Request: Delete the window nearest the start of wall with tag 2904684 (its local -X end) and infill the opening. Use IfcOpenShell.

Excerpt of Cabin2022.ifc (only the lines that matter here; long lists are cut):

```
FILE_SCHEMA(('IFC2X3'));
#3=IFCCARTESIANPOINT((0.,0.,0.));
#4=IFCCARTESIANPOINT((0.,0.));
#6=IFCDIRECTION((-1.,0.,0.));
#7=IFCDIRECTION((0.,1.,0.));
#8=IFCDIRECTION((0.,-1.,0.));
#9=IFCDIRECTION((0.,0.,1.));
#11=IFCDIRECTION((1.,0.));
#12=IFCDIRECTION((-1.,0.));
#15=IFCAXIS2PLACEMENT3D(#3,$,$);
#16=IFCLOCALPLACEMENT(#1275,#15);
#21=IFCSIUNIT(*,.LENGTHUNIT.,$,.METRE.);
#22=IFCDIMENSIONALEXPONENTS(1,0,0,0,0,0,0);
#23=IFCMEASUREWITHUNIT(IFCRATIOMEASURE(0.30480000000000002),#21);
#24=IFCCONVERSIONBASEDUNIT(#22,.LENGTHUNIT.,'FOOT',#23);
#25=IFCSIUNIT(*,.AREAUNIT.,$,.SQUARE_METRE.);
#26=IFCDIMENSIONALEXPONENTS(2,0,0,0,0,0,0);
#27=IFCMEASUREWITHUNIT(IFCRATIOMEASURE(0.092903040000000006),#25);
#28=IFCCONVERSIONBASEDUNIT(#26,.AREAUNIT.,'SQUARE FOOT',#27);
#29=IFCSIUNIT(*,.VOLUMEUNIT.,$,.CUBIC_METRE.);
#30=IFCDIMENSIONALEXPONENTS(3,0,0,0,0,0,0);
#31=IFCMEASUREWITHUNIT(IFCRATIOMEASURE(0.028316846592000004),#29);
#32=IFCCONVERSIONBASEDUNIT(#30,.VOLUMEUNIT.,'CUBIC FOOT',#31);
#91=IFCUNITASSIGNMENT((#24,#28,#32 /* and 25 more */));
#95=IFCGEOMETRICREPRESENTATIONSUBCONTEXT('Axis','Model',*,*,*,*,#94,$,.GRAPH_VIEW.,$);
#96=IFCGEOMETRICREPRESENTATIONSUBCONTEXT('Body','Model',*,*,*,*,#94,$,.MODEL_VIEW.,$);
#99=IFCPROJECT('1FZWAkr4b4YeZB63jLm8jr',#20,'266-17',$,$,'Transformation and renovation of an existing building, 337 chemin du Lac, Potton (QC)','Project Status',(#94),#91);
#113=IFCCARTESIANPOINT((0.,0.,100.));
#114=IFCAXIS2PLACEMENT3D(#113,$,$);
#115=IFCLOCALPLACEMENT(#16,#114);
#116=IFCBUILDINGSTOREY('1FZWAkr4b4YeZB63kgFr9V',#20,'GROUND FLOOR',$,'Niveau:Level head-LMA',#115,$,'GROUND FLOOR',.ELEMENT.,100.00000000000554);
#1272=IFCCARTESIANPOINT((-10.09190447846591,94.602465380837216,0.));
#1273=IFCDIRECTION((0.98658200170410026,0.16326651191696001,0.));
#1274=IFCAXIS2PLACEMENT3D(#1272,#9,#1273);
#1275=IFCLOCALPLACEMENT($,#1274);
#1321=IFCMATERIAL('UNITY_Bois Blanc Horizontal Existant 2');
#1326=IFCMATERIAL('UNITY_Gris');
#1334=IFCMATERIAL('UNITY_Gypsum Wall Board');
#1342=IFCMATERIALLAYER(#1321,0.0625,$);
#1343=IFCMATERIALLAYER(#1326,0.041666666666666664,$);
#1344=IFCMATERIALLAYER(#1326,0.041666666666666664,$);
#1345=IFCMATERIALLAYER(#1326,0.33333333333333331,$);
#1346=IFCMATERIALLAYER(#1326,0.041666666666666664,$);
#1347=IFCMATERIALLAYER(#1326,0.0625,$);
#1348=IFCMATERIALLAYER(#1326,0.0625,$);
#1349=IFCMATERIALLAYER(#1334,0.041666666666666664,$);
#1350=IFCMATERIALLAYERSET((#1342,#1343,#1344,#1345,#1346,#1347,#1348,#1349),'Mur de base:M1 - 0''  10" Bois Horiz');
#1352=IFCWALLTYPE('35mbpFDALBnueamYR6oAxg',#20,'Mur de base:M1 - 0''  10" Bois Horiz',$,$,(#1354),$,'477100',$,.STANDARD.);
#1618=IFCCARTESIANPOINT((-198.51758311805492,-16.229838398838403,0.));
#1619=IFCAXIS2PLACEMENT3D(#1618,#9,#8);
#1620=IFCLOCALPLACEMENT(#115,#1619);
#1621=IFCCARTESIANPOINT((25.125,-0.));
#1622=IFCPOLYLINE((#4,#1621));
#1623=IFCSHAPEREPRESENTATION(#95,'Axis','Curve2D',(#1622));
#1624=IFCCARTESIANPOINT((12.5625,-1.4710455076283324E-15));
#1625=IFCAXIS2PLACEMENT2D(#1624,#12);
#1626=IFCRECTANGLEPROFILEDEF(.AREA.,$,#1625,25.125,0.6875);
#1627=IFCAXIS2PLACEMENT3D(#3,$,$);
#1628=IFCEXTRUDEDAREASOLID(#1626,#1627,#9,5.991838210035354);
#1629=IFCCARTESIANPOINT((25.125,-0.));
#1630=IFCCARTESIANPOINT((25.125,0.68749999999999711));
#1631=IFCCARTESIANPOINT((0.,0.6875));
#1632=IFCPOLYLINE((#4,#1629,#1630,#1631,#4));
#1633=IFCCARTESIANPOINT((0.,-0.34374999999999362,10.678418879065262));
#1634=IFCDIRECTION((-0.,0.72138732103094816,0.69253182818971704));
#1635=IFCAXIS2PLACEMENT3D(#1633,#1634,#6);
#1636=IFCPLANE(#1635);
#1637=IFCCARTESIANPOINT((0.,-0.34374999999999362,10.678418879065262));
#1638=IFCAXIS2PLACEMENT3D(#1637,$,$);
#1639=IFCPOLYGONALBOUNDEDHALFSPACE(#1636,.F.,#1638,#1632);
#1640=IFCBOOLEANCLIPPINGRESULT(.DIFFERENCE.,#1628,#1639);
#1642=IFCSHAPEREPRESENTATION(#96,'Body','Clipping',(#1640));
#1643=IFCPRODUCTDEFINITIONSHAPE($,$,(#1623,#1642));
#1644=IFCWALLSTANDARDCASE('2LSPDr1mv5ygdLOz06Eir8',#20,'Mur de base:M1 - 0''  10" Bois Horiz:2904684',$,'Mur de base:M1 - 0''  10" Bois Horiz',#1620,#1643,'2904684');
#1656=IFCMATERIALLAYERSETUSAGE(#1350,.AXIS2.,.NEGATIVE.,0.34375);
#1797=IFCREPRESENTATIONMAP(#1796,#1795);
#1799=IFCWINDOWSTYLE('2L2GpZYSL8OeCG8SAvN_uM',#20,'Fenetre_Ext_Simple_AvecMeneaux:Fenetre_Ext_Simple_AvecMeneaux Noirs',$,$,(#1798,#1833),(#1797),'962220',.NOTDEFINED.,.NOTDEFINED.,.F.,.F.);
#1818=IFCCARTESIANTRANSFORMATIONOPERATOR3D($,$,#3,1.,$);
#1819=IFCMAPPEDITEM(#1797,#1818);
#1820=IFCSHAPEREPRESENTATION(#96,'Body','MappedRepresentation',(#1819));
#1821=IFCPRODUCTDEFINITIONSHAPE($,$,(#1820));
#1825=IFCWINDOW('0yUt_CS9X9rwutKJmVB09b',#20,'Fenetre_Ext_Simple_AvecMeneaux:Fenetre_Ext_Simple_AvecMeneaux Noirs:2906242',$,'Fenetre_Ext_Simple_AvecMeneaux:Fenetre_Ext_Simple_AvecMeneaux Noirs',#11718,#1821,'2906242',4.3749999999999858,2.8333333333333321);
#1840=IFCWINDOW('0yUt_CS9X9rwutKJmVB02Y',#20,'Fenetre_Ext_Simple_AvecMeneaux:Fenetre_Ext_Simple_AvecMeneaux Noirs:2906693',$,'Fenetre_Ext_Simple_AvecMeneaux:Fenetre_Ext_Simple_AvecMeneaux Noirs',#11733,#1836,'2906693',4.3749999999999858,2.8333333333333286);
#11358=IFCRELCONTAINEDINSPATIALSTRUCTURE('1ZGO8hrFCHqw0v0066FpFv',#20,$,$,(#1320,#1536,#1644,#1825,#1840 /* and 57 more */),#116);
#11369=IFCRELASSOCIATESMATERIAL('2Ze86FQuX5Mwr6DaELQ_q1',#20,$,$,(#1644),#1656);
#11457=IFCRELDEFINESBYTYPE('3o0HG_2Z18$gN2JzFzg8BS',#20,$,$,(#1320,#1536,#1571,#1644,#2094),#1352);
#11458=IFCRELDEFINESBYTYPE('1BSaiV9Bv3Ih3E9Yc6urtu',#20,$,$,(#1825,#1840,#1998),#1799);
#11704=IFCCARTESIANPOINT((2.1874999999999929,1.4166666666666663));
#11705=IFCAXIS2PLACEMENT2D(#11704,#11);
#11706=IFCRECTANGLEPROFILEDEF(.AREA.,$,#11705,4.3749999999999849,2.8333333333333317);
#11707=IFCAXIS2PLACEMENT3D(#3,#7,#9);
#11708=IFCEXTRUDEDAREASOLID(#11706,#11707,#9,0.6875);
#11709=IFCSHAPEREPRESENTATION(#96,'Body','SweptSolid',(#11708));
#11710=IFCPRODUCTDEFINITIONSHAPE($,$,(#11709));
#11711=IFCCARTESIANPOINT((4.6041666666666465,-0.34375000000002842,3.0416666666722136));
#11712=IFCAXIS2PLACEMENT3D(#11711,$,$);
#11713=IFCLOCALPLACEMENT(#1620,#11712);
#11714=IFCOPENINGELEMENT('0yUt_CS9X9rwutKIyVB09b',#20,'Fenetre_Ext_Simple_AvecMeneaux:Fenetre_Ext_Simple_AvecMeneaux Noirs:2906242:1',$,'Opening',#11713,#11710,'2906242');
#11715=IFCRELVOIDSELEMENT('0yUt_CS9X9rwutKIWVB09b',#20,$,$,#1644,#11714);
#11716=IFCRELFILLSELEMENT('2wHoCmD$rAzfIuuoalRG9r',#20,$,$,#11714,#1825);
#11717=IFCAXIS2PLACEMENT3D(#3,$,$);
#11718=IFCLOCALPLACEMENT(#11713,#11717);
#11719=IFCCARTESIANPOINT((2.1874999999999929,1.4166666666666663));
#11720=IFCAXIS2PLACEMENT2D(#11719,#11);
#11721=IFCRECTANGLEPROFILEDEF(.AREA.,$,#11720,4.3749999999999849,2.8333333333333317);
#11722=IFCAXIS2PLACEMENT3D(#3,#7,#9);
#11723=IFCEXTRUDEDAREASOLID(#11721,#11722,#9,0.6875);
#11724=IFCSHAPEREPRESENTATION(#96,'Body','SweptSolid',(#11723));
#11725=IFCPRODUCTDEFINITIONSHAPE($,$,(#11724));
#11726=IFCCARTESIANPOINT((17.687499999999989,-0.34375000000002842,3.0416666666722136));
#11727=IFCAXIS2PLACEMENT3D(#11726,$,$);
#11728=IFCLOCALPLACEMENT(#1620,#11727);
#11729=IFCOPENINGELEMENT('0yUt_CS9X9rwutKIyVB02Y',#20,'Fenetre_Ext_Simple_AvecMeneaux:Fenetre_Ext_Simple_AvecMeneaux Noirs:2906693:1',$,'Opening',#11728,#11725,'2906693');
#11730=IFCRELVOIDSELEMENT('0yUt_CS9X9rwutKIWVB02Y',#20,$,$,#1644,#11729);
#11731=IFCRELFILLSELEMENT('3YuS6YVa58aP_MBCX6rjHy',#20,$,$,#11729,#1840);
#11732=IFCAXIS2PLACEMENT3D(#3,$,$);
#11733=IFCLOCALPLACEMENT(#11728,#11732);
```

```python
import ifcopenshell
import ifcopenshell.api.feature
import ifcopenshell.api.root
import ifcopenshell.geom
import ifcopenshell.util.shape

model = ifcopenshell.open("Cabin2022.ifc")
settings = ifcopenshell.geom.settings()


def volume(element):
    """Net volume in cubic metres, openings subtracted."""
    shape = ifcopenshell.geom.create_shape(settings, element)
    return ifcopenshell.util.shape.get_volume(shape.geometry)


window = model.by_guid("0yUt_CS9X9rwutKJmVB09b")
opening = window.FillsVoids[0].RelatingOpeningElement
wall = opening.VoidsElements[0].RelatingBuildingElement
before = volume(wall)

ifcopenshell.api.root.remove_product(model, product=window)
ifcopenshell.api.feature.remove_feature(model, feature=opening)

after = volume(wall)

print(f"wall volume {before:.3f} -> {after:.3f} m3")

model.write("Cabin2022_rev.ifc")
```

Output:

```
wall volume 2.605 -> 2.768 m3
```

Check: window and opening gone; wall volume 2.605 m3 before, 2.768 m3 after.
